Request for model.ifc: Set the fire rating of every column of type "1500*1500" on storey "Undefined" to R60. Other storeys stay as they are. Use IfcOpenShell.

First a look at what the model holds.

```python
import ifcopenshell
import ifcopenshell.util.element

model = ifcopenshell.open("model.ifc")
print(model.schema)
storey = next(s for s in model.by_type("IfcBuildingStorey") if s.Name == "Undefined")
columns = [e for e in ifcopenshell.util.element.get_decomposition(storey) if e.is_a("IfcColumn")]
seen = {}
for e in columns:
    element_type = ifcopenshell.util.element.get_type(e)
    key = (element_type.Name if element_type != e and element_type else None, ifcopenshell.util.element.get_pset(e, "Pset_ColumnCommon", "FireRating"))
    seen[key] = seen.get(key, 0) + 1
for (name, value), count in sorted(seen.items(), key=str):
    print(count, "x", name, "|", value)
```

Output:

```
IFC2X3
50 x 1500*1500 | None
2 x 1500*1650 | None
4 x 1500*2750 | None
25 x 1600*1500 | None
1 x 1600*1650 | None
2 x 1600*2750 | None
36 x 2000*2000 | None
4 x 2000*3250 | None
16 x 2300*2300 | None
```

```python
import ifcopenshell
import ifcopenshell.api.pset
import ifcopenshell.util.element

model = ifcopenshell.open("model.ifc")

storey = next(s for s in model.by_type("IfcBuildingStorey") if s.Name == "Undefined")
columns = [e for e in ifcopenshell.util.element.get_decomposition(storey) if e.is_a("IfcColumn")]

count = 0
for e in columns:
    element_type = ifcopenshell.util.element.get_type(e)
    if element_type in (None, e) or element_type.Name != "1500*1500":
        continue
    found = ifcopenshell.util.element.get_pset(e, "Pset_ColumnCommon", should_inherit=False)
    if found:
        pset = model.by_id(found["id"])
        if len(ifcopenshell.util.element.get_elements_by_pset(pset)) > 1:
            pset = ifcopenshell.api.pset.unshare_pset(model, products=[e], pset=pset)[0]
    else:
        pset = ifcopenshell.api.pset.add_pset(model, product=e, name="Pset_ColumnCommon")
    ifcopenshell.api.pset.edit_pset(model, pset=pset, properties={"FireRating": "R60"})
    count += 1

print(count, "columns updated")

model.write("model-out.ifc")
```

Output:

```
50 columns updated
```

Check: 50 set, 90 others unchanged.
